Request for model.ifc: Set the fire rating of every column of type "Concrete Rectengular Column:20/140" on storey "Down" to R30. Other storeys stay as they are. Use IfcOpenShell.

First a look at what the model holds.

```python
import ifcopenshell
import ifcopenshell.util.element

model = ifcopenshell.open("model.ifc")
print(model.schema)
storey = next(s for s in model.by_type("IfcBuildingStorey") if s.Name == "Down")
columns = [e for e in ifcopenshell.util.element.get_decomposition(storey) if e.is_a("IfcColumn")]
seen = {}
for e in columns:
    element_type = ifcopenshell.util.element.get_type(e)
    key = (element_type.Name if element_type != e and element_type else None, ifcopenshell.util.element.get_pset(e, "Pset_ColumnCommon", "FireRating"))
    seen[key] = seen.get(key, 0) + 1
for (name, value), count in sorted(seen.items(), key=str):
    print(count, "x", name, "|", value)
```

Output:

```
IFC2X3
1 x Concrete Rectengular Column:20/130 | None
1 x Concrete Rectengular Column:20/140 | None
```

```python
import ifcopenshell
import ifcopenshell.api.pset
import ifcopenshell.util.element

model = ifcopenshell.open("model.ifc")

storey = next(s for s in model.by_type("IfcBuildingStorey") if s.Name == "Down")
columns = [e for e in ifcopenshell.util.element.get_decomposition(storey) if e.is_a("IfcColumn")]

count = 0
for e in columns:
    element_type = ifcopenshell.util.element.get_type(e)
    if element_type in (None, e) or element_type.Name != "Concrete Rectengular Column:20/140":
        continue
    # add_pset returns the element's existing set when there is one.
    pset = ifcopenshell.api.pset.add_pset(model, product=e, name="Pset_ColumnCommon")
    ifcopenshell.api.pset.edit_pset(model, pset=pset, properties={"FireRating": "R30"})
    count += 1

print(count, "columns updated")

model.write("model_rev.ifc")
```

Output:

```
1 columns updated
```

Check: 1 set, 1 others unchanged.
